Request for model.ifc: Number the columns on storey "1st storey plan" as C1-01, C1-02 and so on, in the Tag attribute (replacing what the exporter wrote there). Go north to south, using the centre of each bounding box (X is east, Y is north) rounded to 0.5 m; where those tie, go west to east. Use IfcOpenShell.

First a look at what the model holds.

```python
import ifcopenshell
import ifcopenshell.util.element
import ifcopenshell.util.placement

model = ifcopenshell.open("model.ifc")
print(model.schema)
storey = next(s for s in model.by_type("IfcBuildingStorey") if s.Name == "1st storey plan")
columns = [e for e in ifcopenshell.util.element.get_decomposition(storey) if e.is_a("IfcColumn")]
for e in sorted(columns, key=lambda e: e.id()):
    origin = ifcopenshell.util.placement.get_local_placement(e.ObjectPlacement)[:3, 3]
    print(e.id(), e.Tag, e.Name, origin.round(2) + 0.0, sep=" | ")
```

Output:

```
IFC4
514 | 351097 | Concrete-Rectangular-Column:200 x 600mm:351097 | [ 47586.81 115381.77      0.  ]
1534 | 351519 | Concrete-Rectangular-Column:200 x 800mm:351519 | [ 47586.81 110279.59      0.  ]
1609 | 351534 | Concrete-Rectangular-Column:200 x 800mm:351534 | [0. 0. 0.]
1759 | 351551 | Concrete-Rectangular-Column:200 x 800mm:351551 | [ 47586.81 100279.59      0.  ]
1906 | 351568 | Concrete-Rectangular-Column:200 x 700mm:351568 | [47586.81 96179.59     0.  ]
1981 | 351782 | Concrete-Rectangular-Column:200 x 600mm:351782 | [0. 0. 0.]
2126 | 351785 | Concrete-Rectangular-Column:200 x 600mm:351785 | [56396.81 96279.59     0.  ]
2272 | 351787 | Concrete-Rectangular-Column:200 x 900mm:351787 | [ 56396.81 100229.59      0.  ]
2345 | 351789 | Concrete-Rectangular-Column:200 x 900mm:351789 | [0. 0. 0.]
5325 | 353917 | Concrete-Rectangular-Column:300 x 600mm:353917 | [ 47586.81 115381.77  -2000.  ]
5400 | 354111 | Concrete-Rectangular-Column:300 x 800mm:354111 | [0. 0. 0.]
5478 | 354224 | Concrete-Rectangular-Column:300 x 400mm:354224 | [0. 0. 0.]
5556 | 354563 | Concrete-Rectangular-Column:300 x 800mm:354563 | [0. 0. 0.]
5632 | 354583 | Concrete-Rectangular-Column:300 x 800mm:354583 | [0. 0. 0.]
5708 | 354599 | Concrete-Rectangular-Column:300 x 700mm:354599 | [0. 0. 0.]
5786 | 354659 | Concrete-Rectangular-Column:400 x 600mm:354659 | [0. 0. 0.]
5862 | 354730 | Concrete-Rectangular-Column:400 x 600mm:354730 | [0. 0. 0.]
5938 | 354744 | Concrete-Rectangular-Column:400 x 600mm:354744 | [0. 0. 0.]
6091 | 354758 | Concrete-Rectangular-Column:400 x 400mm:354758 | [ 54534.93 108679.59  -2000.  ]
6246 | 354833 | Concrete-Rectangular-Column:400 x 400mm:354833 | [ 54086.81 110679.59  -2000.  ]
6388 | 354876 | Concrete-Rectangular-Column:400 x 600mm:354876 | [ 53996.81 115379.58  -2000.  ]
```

```python
import ifcopenshell
import ifcopenshell.geom
import ifcopenshell.util.element
import ifcopenshell.util.shape

model = ifcopenshell.open("model.ifc")
settings = ifcopenshell.geom.settings()
settings.set("use-world-coords", True)


def centre(element):
    shape = ifcopenshell.geom.create_shape(settings, element)
    return ifcopenshell.util.shape.get_bbox_centroid(shape.geometry)


storey = next(s for s in model.by_type("IfcBuildingStorey") if s.Name == "1st storey plan")
columns = [e for e in ifcopenshell.util.element.get_decomposition(storey) if e.is_a("IfcColumn")]

# Insertion points can sit at a corner or the storey origin, so sort by the geometry (in metres).
centres = {e: centre(e) for e in columns}
columns.sort(key=lambda e: (-round(centres[e][1] / 0.5), centres[e][0]))

for i, e in enumerate(columns, start=1):
    number = f"C1-{i:02d}"
    e.Tag = number
    print(e.id(), number)

model.write("model-out.ifc")
```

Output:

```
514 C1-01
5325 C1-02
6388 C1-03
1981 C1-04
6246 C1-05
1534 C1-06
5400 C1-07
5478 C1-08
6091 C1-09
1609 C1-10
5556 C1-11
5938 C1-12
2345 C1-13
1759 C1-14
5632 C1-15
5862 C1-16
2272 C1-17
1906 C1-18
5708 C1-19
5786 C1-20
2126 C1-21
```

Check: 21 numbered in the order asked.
